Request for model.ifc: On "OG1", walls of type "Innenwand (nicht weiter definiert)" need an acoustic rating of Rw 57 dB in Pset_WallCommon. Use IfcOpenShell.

First a look at what the model holds.

```python
import ifcopenshell
import ifcopenshell.util.element

model = ifcopenshell.open("model.ifc")
print(model.schema)
storey = next(s for s in model.by_type("IfcBuildingStorey") if s.Name == "OG1")
walls = [e for e in ifcopenshell.util.element.get_decomposition(storey) if e.is_a("IfcWall")]
seen = {}
for e in walls:
    element_type = ifcopenshell.util.element.get_type(e)
    key = (element_type.Name if element_type != e and element_type else None, ifcopenshell.util.element.get_pset(e, "Pset_WallCommon", "AcousticRating"))
    seen[key] = seen.get(key, 0) + 1
for (name, value), count in sorted(seen.items(), key=str):
    print(count, "x", name, "|", value)
```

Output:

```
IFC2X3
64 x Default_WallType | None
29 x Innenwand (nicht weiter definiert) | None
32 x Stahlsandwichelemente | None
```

```python
import ifcopenshell
import ifcopenshell.api.pset
import ifcopenshell.util.element

model = ifcopenshell.open("model.ifc")

storey = next(s for s in model.by_type("IfcBuildingStorey") if s.Name == "OG1")
walls = [e for e in ifcopenshell.util.element.get_decomposition(storey) if e.is_a("IfcWall")]

count = 0
for e in walls:
    element_type = ifcopenshell.util.element.get_type(e)
    if element_type in (None, e) or element_type.Name != "Innenwand (nicht weiter definiert)":
        continue
    # add_pset returns the element's existing set when there is one.
    pset = ifcopenshell.api.pset.add_pset(model, product=e, name="Pset_WallCommon")
    ifcopenshell.api.pset.edit_pset(model, pset=pset, properties={"AcousticRating": "Rw 57 dB"})
    count += 1

print(count, "walls updated")

model.write("model_updated.ifc")
```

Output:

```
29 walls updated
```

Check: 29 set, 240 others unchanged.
